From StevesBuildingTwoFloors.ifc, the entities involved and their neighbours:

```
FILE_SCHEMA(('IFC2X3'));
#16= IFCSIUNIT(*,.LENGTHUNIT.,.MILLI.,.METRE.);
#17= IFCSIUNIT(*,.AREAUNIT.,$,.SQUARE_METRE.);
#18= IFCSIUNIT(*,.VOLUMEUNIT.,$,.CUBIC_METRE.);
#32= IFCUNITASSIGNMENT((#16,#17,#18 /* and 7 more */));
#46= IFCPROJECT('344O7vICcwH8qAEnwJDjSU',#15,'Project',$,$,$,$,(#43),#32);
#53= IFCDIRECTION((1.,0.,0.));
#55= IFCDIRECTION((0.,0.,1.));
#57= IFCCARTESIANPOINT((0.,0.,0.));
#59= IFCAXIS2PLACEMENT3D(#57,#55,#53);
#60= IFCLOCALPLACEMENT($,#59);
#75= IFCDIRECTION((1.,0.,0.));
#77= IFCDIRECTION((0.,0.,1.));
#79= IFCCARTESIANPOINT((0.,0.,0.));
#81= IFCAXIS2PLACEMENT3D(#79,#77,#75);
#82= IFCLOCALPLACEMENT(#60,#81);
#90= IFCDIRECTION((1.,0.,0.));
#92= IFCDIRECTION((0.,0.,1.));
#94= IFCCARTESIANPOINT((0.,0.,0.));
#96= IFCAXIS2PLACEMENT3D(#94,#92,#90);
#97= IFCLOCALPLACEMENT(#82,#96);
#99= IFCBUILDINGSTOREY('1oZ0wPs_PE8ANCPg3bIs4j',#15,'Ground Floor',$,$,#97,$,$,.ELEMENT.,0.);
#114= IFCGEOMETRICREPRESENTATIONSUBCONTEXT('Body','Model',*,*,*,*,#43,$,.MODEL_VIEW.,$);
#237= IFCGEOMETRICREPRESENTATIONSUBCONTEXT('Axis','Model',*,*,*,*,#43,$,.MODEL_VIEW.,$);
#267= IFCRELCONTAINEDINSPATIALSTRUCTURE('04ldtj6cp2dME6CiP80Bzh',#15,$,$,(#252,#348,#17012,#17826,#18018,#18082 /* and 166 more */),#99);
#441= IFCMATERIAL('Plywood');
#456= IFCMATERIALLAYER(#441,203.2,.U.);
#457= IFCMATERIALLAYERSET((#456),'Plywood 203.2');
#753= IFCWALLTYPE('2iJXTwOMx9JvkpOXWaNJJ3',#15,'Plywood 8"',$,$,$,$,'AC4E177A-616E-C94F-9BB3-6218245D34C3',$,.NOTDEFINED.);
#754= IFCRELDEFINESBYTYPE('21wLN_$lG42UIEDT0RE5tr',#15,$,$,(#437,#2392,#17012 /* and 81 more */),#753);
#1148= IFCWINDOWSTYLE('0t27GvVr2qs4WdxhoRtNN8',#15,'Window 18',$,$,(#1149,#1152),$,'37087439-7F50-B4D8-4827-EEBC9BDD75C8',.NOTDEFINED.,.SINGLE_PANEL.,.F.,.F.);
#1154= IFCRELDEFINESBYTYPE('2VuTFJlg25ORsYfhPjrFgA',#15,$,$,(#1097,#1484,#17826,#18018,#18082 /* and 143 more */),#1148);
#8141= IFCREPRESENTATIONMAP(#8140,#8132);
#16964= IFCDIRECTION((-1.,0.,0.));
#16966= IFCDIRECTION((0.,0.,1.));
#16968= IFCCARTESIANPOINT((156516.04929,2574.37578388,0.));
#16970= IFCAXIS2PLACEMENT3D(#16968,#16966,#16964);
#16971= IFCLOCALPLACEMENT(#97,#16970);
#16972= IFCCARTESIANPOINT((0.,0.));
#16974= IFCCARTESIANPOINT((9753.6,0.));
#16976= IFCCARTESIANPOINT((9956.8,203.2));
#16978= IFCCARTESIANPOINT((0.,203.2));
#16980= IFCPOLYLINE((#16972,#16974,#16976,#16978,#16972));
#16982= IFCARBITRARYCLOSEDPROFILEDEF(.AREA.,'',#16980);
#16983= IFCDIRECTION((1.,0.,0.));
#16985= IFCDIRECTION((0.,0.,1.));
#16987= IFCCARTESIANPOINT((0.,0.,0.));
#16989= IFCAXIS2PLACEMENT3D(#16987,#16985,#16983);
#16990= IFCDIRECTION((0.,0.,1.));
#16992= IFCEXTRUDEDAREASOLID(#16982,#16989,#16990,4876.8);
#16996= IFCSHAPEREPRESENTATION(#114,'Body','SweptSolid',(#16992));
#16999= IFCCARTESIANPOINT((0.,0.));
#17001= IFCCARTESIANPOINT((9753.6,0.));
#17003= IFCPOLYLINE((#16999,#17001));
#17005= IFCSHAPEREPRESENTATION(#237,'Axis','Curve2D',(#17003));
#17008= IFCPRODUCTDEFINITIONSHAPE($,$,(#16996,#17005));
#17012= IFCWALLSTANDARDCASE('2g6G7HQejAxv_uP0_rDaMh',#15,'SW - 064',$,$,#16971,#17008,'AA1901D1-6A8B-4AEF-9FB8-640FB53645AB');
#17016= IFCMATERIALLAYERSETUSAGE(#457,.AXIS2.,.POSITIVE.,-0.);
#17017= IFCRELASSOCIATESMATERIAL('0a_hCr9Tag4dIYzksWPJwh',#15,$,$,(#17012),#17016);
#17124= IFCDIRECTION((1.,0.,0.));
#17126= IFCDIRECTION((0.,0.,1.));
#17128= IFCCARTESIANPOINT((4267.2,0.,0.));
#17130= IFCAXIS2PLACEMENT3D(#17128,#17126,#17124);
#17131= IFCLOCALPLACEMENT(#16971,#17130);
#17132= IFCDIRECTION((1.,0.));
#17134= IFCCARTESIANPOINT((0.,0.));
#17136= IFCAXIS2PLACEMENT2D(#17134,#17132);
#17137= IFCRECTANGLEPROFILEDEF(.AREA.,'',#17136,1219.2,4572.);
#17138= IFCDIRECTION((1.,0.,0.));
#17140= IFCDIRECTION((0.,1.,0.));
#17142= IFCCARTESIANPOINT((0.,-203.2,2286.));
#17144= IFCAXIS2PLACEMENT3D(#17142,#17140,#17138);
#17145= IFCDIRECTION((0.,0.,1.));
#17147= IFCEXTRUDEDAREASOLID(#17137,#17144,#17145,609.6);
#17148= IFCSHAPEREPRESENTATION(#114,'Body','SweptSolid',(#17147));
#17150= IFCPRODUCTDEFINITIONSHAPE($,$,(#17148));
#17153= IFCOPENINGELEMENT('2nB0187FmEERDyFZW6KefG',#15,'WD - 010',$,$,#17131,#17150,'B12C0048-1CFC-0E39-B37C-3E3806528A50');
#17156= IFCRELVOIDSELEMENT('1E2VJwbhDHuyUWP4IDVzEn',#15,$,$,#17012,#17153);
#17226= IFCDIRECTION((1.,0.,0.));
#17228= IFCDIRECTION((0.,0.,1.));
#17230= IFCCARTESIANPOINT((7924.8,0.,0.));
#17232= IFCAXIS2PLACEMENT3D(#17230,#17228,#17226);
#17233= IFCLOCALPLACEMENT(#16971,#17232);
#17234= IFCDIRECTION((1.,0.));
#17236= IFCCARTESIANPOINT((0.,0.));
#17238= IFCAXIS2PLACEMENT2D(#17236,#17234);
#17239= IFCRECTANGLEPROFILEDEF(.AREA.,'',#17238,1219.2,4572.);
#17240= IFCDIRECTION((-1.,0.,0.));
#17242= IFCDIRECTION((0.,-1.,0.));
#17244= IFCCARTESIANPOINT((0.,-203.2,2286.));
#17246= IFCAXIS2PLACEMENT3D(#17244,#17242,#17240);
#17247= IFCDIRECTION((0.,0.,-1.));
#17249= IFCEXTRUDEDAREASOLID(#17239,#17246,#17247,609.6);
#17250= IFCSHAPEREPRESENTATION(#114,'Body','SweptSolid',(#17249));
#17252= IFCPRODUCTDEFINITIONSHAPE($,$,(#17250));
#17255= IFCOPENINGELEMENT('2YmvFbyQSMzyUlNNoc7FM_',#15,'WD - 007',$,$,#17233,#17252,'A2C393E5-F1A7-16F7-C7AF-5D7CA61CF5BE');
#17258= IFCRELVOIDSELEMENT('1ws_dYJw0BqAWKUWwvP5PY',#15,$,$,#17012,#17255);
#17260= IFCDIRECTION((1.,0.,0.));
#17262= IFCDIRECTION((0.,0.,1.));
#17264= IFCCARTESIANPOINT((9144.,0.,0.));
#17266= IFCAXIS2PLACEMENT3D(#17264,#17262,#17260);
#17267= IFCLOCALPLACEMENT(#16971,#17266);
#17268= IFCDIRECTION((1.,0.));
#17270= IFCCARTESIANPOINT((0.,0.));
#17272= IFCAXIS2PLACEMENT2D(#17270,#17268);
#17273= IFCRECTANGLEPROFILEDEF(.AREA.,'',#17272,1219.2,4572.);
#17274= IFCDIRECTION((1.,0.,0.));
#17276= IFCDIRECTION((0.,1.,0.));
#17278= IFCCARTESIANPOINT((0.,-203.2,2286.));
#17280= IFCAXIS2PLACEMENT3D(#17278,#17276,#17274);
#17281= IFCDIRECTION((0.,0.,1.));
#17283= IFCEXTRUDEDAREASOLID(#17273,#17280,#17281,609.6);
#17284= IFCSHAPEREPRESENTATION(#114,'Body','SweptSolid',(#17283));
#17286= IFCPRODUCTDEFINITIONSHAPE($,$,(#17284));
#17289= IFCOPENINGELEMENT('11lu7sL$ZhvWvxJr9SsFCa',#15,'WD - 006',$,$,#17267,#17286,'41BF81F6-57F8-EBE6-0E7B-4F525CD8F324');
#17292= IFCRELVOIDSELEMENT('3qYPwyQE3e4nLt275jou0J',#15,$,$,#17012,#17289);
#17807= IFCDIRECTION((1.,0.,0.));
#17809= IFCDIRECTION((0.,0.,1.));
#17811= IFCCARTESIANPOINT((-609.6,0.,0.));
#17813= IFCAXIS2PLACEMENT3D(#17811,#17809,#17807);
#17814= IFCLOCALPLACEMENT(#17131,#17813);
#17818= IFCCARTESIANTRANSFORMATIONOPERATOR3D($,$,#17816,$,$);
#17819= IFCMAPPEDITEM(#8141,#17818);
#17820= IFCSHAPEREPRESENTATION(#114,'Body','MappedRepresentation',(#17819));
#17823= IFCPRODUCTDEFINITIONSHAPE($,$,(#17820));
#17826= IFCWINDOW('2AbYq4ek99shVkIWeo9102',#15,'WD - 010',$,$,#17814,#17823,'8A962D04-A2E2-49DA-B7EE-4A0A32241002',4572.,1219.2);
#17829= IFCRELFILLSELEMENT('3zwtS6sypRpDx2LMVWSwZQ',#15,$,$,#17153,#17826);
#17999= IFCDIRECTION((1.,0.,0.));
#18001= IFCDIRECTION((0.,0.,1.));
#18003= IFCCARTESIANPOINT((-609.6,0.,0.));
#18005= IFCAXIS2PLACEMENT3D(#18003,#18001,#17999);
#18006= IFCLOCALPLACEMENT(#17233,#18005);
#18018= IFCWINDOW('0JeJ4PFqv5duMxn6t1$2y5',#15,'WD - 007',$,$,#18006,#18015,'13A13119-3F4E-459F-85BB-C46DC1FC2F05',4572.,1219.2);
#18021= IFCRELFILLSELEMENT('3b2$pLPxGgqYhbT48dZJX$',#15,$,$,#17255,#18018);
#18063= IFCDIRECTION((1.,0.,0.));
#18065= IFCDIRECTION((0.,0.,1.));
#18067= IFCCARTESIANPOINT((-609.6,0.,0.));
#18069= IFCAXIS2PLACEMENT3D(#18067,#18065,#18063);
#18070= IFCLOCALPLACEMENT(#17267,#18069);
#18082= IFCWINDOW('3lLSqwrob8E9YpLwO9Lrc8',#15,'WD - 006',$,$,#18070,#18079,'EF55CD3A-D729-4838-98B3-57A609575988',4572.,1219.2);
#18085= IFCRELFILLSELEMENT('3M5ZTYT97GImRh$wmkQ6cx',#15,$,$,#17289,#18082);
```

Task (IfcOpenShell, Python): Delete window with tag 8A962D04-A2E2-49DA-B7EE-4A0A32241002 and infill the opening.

```python
import ifcopenshell
import ifcopenshell.api.feature
import ifcopenshell.api.root
import ifcopenshell.geom
import ifcopenshell.util.shape

model = ifcopenshell.open("StevesBuildingTwoFloors.ifc")
settings = ifcopenshell.geom.settings()


def volume(element):
    """Net volume in cubic metres, openings subtracted."""
    shape = ifcopenshell.geom.create_shape(settings, element)
    return ifcopenshell.util.shape.get_volume(shape.geometry)


window = model.by_guid("2AbYq4ek99shVkIWeo9102")
opening = window.FillsVoids[0].RelatingOpeningElement
wall = opening.VoidsElements[0].RelatingBuildingElement
before = volume(wall)

ifcopenshell.api.root.remove_product(model, product=window)
ifcopenshell.api.feature.remove_feature(model, feature=opening)

after = volume(wall)

print(f"wall volume {before:.3f} -> {after:.3f} m3")

model.write("StevesBuildingTwoFloors_rev.ifc")
```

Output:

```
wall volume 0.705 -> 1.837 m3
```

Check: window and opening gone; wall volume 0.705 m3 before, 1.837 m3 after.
